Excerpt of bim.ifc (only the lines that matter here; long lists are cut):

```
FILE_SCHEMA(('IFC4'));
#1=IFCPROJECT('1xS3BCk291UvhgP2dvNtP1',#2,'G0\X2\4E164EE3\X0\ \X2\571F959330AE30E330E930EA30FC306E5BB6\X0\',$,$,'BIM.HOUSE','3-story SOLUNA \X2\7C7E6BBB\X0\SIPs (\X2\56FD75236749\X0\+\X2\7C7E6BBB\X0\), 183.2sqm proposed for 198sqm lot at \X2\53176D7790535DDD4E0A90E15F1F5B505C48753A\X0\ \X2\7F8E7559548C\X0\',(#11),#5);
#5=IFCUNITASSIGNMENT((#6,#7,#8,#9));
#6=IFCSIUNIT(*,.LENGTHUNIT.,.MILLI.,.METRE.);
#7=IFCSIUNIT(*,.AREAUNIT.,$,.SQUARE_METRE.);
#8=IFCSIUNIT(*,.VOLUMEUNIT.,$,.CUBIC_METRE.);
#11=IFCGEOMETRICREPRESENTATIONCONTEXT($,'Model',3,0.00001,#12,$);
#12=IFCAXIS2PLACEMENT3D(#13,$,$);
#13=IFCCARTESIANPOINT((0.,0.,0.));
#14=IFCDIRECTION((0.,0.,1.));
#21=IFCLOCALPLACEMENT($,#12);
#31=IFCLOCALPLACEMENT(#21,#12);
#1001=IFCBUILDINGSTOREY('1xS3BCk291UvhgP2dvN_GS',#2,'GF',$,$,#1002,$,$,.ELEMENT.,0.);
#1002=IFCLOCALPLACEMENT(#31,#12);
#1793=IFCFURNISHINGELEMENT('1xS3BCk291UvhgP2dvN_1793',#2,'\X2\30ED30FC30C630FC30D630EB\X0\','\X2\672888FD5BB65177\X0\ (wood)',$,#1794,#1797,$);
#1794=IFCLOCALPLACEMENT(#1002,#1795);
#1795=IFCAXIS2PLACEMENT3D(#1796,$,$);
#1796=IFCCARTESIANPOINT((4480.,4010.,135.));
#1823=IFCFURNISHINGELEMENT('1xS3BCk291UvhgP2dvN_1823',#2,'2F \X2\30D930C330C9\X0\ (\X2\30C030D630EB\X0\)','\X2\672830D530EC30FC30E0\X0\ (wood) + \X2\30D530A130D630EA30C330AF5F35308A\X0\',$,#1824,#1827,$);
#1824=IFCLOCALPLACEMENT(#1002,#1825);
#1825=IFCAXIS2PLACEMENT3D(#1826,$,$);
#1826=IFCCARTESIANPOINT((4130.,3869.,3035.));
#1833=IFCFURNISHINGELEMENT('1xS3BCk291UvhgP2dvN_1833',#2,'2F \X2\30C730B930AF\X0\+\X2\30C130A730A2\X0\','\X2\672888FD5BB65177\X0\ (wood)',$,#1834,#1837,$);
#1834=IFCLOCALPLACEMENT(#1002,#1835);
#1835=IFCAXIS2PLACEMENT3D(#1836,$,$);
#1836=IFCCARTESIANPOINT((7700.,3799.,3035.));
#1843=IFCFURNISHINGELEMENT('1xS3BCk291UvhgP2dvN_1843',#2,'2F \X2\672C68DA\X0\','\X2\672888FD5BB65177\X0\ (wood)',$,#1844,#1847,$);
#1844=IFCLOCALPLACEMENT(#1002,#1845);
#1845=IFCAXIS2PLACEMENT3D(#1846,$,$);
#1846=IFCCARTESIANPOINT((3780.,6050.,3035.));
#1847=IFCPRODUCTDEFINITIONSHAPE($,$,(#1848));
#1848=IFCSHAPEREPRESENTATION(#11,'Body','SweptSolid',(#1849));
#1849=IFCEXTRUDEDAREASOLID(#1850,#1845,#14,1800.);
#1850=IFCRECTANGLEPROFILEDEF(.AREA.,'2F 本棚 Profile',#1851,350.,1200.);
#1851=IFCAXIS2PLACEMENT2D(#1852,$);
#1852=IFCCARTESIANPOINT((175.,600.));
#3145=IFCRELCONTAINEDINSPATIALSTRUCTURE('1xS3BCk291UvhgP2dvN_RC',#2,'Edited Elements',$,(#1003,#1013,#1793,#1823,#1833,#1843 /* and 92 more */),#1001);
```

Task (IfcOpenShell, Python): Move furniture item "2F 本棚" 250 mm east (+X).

```python
import ifcopenshell
import ifcopenshell.api.geometry
import ifcopenshell.util.placement
import ifcopenshell.util.unit

model = ifcopenshell.open("bim.ifc")
unit_scale = ifcopenshell.util.unit.calculate_unit_scale(model)

item = model.by_guid("1xS3BCk291UvhgP2dvN_1843")
matrix = ifcopenshell.util.placement.get_local_placement(item.ObjectPlacement)
matrix[0, 3] += 0.25 / unit_scale
ifcopenshell.api.geometry.edit_object_placement(model, product=item, matrix=matrix, is_si=False)

print(ifcopenshell.util.placement.get_local_placement(item.ObjectPlacement).round(3) + 0.0)

model.write("bim_rev.ifc")
```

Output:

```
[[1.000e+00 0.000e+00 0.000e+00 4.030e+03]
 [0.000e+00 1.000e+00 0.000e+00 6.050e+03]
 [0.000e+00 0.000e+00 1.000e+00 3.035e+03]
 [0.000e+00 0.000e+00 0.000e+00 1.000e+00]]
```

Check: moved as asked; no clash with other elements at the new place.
